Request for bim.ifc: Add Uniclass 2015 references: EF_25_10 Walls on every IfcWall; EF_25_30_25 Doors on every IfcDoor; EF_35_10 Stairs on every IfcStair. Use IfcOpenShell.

First a look at what the model holds.

```python
import ifcopenshell

model = ifcopenshell.open("bim.ifc")
print(model.schema)
print("classifications:", [c.Name for c in model.by_type("IfcClassification")])
for ifc_class in ("IfcDoor", "IfcRoof", "IfcStair", "IfcWall", "IfcWindow"):
    print(ifc_class, len(model.by_type(ifc_class)))
```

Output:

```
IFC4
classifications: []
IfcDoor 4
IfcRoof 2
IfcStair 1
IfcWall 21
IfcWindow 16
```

```python
import ifcopenshell
import ifcopenshell.api.classification

model = ifcopenshell.open("bim.ifc")

system = ifcopenshell.api.classification.add_classification(model, classification="Uniclass 2015")

codes = {
    "IfcWall": ("EF_25_10", "Walls"),
    "IfcDoor": ("EF_25_30_25", "Doors"),
    "IfcStair": ("EF_35_10", "Stairs"),
}
for ifc_class, (code, name) in codes.items():
    products = model.by_type(ifc_class)
    ifcopenshell.api.classification.add_reference(
        model, products=products, classification=system, identification=code, name=name
    )
    print(code, len(products))

model.write("bim_v2.ifc")
```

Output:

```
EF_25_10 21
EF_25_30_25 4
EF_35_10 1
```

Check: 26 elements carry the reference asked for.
